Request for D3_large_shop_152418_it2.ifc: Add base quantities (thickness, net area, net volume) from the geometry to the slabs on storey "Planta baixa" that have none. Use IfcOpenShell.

First a look at what the model holds.

```python
import ifcopenshell
import ifcopenshell.util.element
import ifcopenshell.util.unit

model = ifcopenshell.open("D3_large_shop_152418_it2.ifc")
print(model.schema)
for unit_type in ("LENGTHUNIT", "AREAUNIT", "VOLUMEUNIT"):
    print(unit_type, ifcopenshell.util.unit.calculate_unit_scale(model, unit_type))
storey = next(s for s in model.by_type("IfcBuildingStorey") if s.Name == "Planta baixa")
slabs = [e for e in ifcopenshell.util.element.get_decomposition(storey) if e.is_a("IfcSlab")]
for e in sorted(slabs, key=lambda e: e.id()):
    print(e.id(), e.is_a(), e.Name, list(ifcopenshell.util.element.get_psets(e, qtos_only=True)), sep=" | ")
```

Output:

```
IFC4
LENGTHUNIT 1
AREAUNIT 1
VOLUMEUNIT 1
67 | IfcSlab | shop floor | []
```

```python
import ifcopenshell
import ifcopenshell.api.pset
import ifcopenshell.geom
import ifcopenshell.util.element
import ifcopenshell.util.shape
import ifcopenshell.util.unit

model = ifcopenshell.open("D3_large_shop_152418_it2.ifc")
unit_scale = ifcopenshell.util.unit.calculate_unit_scale(model)
area_scale = ifcopenshell.util.unit.calculate_unit_scale(model, "AREAUNIT")
volume_scale = ifcopenshell.util.unit.calculate_unit_scale(model, "VOLUMEUNIT")
settings = ifcopenshell.geom.settings()

storey = next(s for s in model.by_type("IfcBuildingStorey") if s.Name == "Planta baixa")
slabs = [e for e in ifcopenshell.util.element.get_decomposition(storey) if e.is_a("IfcSlab")]

for e in sorted(slabs, key=lambda e: e.id()):
    if ifcopenshell.util.element.get_psets(e, qtos_only=True, should_inherit=False):
        continue
    # Geometry comes back in metres, in the element's own axes.
    shape = ifcopenshell.geom.create_shape(settings, e)
    values = {
        "Width": ifcopenshell.util.shape.get_z(shape.geometry) / unit_scale,
        "NetArea": ifcopenshell.util.shape.get_footprint_area(shape.geometry) / area_scale,
        "NetVolume": ifcopenshell.util.shape.get_volume(shape.geometry) / volume_scale,
    }
    qto = ifcopenshell.api.pset.add_qto(model, product=e, name="Qto_SlabBaseQuantities")
    ifcopenshell.api.pset.edit_qto(model, qto=qto, properties=values)
    print(e.id(), {k: round(v, 3) for k, v in values.items()})

model.write("D3_large_shop_152418_it2-out.ifc")
```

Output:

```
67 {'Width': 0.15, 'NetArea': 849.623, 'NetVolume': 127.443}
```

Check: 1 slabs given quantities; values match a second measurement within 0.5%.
